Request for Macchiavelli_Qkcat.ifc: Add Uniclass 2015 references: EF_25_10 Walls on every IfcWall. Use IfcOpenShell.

First a look at what the model holds.

```python
import ifcopenshell

model = ifcopenshell.open("Macchiavelli_Qkcat.ifc")
print(model.schema)
print("classifications:", [c.Name for c in model.by_type("IfcClassification")])
for ifc_class in ("IfcDoor", "IfcRoof", "IfcStair", "IfcWall", "IfcWindow"):
    print(ifc_class, len(model.by_type(ifc_class)))
```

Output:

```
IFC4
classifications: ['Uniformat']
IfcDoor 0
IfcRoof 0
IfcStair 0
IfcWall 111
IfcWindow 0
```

```python
import ifcopenshell
import ifcopenshell.api.classification

model = ifcopenshell.open("Macchiavelli_Qkcat.ifc")

system = ifcopenshell.api.classification.add_classification(model, classification="Uniclass 2015")

codes = {
    "IfcWall": ("EF_25_10", "Walls"),
}
for ifc_class, (code, name) in codes.items():
    products = model.by_type(ifc_class)
    ifcopenshell.api.classification.add_reference(
        model, products=products, classification=system, identification=code, name=name
    )
    print(code, len(products))

model.write("Macchiavelli_Qkcat-out.ifc")
```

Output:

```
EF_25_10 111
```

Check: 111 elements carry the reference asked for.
